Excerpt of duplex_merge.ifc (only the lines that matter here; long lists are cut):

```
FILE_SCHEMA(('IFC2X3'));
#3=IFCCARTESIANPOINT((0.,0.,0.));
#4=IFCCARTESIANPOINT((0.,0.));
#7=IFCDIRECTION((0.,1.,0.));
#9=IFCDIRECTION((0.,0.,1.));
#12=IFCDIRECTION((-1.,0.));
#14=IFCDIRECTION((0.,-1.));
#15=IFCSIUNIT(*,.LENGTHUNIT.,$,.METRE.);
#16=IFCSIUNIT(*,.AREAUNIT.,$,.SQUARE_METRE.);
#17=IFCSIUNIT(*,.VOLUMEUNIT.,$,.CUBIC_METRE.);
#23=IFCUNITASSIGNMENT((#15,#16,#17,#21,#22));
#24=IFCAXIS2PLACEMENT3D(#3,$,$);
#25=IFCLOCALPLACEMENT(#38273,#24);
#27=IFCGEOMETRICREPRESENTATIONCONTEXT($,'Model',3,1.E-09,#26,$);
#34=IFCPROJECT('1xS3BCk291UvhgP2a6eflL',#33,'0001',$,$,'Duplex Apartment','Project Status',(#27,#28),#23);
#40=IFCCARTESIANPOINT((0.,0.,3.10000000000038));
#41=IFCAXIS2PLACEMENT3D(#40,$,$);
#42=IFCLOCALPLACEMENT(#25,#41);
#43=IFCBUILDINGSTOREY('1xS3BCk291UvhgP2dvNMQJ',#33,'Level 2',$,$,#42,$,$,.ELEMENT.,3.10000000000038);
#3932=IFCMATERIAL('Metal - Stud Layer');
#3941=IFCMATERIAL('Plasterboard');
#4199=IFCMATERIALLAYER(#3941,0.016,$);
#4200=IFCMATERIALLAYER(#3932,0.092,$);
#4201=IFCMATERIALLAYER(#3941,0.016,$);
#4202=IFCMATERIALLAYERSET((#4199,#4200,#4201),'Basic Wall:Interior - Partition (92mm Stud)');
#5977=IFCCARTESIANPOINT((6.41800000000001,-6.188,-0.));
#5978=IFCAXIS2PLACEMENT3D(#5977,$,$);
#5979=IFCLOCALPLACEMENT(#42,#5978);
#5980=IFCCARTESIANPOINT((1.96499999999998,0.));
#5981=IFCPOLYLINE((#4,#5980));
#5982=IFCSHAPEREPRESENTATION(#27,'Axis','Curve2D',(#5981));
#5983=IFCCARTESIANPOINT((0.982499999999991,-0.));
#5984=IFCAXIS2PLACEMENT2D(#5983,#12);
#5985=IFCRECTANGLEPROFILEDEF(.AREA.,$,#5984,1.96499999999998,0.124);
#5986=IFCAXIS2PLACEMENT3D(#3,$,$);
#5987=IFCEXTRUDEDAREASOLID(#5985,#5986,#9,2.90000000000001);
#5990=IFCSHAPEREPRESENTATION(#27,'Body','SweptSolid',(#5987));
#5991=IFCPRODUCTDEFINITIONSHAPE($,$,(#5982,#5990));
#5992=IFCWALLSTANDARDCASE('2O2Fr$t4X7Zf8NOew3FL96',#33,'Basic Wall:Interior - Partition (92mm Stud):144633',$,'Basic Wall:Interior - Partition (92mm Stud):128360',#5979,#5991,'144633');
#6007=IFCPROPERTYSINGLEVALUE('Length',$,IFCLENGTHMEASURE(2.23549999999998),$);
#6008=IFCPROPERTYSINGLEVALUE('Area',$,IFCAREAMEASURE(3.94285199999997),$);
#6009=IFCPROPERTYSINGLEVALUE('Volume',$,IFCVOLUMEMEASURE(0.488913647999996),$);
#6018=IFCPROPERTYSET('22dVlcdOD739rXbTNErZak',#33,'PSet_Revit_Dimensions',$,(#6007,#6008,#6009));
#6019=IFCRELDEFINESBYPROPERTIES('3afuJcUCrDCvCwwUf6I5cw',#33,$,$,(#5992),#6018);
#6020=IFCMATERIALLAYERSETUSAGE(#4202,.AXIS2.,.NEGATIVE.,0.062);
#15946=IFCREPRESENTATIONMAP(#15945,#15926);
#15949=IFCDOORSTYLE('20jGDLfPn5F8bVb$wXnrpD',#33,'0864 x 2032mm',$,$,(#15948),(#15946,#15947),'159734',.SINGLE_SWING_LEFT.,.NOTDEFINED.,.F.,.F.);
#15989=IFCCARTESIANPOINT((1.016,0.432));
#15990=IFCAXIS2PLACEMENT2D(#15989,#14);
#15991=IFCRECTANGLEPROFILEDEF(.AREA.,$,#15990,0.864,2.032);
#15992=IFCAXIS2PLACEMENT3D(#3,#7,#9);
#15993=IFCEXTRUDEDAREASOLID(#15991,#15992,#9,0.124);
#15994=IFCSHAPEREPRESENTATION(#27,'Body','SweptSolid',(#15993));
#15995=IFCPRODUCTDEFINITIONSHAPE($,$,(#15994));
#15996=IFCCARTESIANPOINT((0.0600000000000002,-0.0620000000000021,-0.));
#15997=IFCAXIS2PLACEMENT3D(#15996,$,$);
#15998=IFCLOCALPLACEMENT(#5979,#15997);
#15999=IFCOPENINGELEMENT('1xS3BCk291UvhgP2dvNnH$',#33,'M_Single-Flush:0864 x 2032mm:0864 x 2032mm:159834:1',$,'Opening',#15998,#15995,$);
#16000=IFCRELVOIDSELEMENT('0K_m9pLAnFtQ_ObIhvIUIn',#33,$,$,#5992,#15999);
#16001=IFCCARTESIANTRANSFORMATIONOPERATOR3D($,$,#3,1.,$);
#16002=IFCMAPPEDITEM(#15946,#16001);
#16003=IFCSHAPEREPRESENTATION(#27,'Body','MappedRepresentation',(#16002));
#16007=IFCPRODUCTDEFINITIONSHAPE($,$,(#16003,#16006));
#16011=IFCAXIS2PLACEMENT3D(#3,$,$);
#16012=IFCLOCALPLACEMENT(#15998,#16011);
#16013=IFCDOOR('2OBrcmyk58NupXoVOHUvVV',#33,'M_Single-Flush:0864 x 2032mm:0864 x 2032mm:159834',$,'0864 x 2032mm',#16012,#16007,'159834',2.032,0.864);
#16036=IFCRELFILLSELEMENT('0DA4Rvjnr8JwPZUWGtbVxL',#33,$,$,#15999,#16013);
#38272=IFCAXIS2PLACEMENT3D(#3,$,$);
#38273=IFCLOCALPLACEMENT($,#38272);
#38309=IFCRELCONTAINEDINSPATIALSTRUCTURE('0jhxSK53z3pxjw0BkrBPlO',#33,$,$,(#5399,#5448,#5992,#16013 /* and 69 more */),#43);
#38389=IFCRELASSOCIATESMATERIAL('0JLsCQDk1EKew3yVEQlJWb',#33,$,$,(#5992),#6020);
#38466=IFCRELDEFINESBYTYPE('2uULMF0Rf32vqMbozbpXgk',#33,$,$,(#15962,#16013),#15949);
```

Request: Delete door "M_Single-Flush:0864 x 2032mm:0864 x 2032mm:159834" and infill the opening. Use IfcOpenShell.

```python
import ifcopenshell
import ifcopenshell.api.feature
import ifcopenshell.api.pset
import ifcopenshell.api.root
import ifcopenshell.geom
import ifcopenshell.util.element
import ifcopenshell.util.shape
import ifcopenshell.util.unit

model = ifcopenshell.open("duplex_merge.ifc")
area_scale = ifcopenshell.util.unit.calculate_unit_scale(model, "AREAUNIT")
volume_scale = ifcopenshell.util.unit.calculate_unit_scale(model, "VOLUMEUNIT")
settings = ifcopenshell.geom.settings()


def volume(element):
    """Net volume in cubic metres, openings subtracted."""
    shape = ifcopenshell.geom.create_shape(settings, element)
    return ifcopenshell.util.shape.get_volume(shape.geometry)


door = model.by_guid("2OBrcmyk58NupXoVOHUvVV")
opening = door.FillsVoids[0].RelatingOpeningElement
wall = opening.VoidsElements[0].RelatingBuildingElement
before = volume(wall)

ifcopenshell.api.root.remove_product(model, product=door)
ifcopenshell.api.feature.remove_feature(model, feature=opening)

after = volume(wall)
thickness = 0.124  # wall thickness in metres

# Update the wall's stored quantities.
pset = model.by_id(ifcopenshell.util.element.get_pset(wall, "PSet_Revit_Dimensions", should_inherit=False)["id"])
ifcopenshell.api.pset.edit_pset(model, pset=pset, properties={
    "Area": model.create_entity("IfcAreaMeasure", after / thickness / area_scale),
    "Volume": model.create_entity("IfcVolumeMeasure", after / volume_scale),
})

print(f"wall volume {before:.3f} -> {after:.3f} m3")

model.write("duplex_merge_rev.ifc")
```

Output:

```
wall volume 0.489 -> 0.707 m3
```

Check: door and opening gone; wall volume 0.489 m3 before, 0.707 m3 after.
